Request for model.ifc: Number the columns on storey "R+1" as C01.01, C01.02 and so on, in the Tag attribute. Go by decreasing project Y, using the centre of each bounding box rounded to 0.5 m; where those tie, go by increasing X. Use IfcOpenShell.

First a look at what the model holds.

```python
import ifcopenshell
import ifcopenshell.util.element
import ifcopenshell.util.placement

model = ifcopenshell.open("model.ifc")
print(model.schema)
storey = next(s for s in model.by_type("IfcBuildingStorey") if s.Name == "R+1")
columns = [e for e in ifcopenshell.util.element.get_decomposition(storey) if e.is_a("IfcColumn")]
for e in sorted(columns, key=lambda e: e.id()):
    origin = ifcopenshell.util.placement.get_local_placement(e.ObjectPlacement)[:3, 3]
    print(e.id(), e.Tag, e.Name, origin.round(2) + 0.0, sep=" | ")
```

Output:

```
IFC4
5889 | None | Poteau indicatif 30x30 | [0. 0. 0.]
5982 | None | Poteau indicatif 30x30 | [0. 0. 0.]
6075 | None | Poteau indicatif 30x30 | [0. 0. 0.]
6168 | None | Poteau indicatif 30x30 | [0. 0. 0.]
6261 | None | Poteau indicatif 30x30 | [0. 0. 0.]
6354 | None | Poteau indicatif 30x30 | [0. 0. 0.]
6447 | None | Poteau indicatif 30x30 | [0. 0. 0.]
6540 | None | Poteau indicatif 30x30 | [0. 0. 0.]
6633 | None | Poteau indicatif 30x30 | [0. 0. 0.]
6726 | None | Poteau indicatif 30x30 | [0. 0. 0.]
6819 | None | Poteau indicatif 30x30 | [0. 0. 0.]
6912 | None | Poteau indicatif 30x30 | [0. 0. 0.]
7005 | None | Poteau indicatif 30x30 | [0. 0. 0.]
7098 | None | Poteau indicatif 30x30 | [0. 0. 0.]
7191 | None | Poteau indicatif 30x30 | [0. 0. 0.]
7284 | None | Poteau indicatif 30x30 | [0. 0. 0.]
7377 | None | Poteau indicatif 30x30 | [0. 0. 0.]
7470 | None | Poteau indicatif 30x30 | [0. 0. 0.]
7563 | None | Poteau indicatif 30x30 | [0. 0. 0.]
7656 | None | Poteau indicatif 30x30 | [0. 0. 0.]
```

```python
import ifcopenshell
import ifcopenshell.geom
import ifcopenshell.util.element
import ifcopenshell.util.shape

model = ifcopenshell.open("model.ifc")
settings = ifcopenshell.geom.settings()
settings.set("use-world-coords", True)


def centre(element):
    shape = ifcopenshell.geom.create_shape(settings, element)
    return ifcopenshell.util.shape.get_bbox_centroid(shape.geometry)


storey = next(s for s in model.by_type("IfcBuildingStorey") if s.Name == "R+1")
columns = [e for e in ifcopenshell.util.element.get_decomposition(storey) if e.is_a("IfcColumn")]

# Insertion points can sit at a corner or the storey origin, so sort by the geometry (in metres).
centres = {e: centre(e) for e in columns}
columns.sort(key=lambda e: (-round(centres[e][1] / 0.5), centres[e][0]))

for i, e in enumerate(columns, start=1):
    number = f"C01.{i:02d}"
    e.Tag = number
    print(e.id(), number)

model.write("model_v2.ifc")
```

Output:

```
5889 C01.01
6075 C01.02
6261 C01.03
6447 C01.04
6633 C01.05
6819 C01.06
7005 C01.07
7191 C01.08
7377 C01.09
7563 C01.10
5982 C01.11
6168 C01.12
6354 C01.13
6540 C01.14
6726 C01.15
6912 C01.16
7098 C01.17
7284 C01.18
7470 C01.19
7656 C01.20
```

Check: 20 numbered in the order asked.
